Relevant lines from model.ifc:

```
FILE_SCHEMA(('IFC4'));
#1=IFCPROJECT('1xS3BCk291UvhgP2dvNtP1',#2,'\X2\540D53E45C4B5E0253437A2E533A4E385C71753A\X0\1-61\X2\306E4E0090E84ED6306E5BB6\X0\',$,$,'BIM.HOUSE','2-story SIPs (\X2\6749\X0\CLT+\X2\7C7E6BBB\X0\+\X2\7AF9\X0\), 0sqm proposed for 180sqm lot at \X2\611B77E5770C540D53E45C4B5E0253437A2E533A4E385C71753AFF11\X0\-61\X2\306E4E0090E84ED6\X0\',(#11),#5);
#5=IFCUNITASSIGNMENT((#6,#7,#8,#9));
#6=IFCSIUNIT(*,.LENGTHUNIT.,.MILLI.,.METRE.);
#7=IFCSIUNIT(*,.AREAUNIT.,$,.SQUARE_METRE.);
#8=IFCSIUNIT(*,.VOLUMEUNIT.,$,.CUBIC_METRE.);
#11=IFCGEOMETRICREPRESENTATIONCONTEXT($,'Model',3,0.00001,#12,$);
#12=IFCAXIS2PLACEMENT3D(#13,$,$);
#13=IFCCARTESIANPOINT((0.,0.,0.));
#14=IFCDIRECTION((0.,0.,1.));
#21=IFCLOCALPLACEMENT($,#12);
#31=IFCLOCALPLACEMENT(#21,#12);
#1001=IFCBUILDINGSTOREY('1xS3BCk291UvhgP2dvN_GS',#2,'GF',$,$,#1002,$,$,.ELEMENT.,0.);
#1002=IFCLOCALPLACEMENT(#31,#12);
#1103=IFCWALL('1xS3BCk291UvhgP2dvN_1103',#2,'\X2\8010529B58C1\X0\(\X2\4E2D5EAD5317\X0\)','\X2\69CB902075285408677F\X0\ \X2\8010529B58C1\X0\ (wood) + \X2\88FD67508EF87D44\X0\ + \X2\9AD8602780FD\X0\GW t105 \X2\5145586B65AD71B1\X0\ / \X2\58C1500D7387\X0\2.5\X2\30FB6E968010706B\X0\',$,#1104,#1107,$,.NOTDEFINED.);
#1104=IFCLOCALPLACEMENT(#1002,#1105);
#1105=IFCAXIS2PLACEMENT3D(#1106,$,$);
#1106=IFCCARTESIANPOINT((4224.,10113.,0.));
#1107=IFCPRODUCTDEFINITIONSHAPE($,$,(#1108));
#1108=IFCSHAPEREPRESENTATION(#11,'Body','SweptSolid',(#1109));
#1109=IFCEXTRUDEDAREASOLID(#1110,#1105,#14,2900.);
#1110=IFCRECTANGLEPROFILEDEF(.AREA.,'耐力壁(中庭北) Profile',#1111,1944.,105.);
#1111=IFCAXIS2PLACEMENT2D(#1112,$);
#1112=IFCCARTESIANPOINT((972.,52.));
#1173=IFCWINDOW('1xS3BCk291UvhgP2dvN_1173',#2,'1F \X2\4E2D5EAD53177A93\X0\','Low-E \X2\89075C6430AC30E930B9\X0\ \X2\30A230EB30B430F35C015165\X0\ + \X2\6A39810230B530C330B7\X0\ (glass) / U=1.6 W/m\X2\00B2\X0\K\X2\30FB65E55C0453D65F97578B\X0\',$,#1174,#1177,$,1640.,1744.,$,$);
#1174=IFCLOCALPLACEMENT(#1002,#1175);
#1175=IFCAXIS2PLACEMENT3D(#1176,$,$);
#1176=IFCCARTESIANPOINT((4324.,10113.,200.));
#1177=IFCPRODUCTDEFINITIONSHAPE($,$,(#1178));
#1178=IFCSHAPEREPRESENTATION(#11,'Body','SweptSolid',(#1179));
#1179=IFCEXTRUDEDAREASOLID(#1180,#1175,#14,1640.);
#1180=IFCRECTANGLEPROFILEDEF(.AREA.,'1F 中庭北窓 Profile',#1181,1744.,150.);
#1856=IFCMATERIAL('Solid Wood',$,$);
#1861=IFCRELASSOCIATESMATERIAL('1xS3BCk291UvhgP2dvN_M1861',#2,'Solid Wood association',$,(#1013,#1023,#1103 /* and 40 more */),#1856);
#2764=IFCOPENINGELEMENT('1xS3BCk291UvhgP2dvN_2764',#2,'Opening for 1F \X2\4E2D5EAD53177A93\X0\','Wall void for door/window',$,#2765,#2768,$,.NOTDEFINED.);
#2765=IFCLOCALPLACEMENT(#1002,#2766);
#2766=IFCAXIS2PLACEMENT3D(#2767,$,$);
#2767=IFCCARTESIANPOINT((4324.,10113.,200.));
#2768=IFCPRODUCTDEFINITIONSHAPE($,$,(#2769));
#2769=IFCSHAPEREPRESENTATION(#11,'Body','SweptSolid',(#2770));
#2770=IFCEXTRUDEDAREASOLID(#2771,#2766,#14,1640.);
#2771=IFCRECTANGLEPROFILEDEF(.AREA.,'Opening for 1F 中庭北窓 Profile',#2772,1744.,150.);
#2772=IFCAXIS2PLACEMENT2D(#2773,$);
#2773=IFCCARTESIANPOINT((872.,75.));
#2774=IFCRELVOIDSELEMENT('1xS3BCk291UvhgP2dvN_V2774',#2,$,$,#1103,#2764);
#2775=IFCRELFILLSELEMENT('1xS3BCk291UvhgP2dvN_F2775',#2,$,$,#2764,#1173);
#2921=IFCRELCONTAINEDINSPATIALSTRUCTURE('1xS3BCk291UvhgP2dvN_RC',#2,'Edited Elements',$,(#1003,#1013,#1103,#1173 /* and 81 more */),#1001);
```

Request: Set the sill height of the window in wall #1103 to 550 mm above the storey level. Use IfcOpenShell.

```python
import numpy as np
import ifcopenshell
import ifcopenshell.api.geometry
import ifcopenshell.geom
import ifcopenshell.util.element
import ifcopenshell.util.placement
import ifcopenshell.util.shape
import ifcopenshell.util.unit

model = ifcopenshell.open("model.ifc")
unit_scale = ifcopenshell.util.unit.calculate_unit_scale(model)

window = model.by_guid("1xS3BCk291UvhgP2dvN_1173")
opening = window.FillsVoids[0].RelatingOpeningElement
storey = ifcopenshell.util.element.get_container(window, ifc_class="IfcBuildingStorey")
level = ifcopenshell.util.placement.get_local_placement(storey.ObjectPlacement)[2, 3]

# The opening's origin need not be at the sill, so measure its lowest point.
shape = ifcopenshell.geom.create_shape(ifcopenshell.geom.settings(), opening)
bottom = ifcopenshell.util.shape.get_shape_bottom_elevation(shape, shape.geometry) / unit_scale
dz = level + 550.0 - bottom

shift = np.array([0.0, 0.0, dz])
# The window is not placed relative to its opening, so move both.
for product in (opening, window):
    matrix = ifcopenshell.util.placement.get_local_placement(product.ObjectPlacement)
    matrix[:3, 3] += shift
    ifcopenshell.api.geometry.edit_object_placement(model, product=product, matrix=matrix, is_si=False)

print(f"moved by {dz * unit_scale:+.3f} m")

model.write("model_updated.ifc")
```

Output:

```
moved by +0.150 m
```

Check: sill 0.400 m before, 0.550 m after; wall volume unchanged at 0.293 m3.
